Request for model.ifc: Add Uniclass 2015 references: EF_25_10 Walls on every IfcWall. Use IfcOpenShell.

First a look at what the model holds.

```python
import ifcopenshell

model = ifcopenshell.open("model.ifc")
print(model.schema)
print("classifications:", [c.Name for c in model.by_type("IfcClassification")])
for ifc_class in ("IfcDoor", "IfcRoof", "IfcStair", "IfcWall", "IfcWindow"):
    print(ifc_class, len(model.by_type(ifc_class)))
```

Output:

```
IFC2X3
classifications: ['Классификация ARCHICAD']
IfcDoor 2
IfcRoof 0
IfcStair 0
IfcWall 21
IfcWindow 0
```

```python
import ifcopenshell
import ifcopenshell.api.classification

model = ifcopenshell.open("model.ifc")

# IFC2X3 requires Source and Edition and has no link from the project to the system.
system = model.create_entity("IfcClassification", Source="NBS", Edition="2015", Name="Uniclass 2015")

codes = {
    "IfcWall": ("EF_25_10", "Walls"),
}
for ifc_class, (code, name) in codes.items():
    products = model.by_type(ifc_class)
    ifcopenshell.api.classification.add_reference(
        model, products=products, classification=system, identification=code, name=name
    )
    print(code, len(products))

model.write("model_edited.ifc")
```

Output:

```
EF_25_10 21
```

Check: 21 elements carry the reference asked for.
